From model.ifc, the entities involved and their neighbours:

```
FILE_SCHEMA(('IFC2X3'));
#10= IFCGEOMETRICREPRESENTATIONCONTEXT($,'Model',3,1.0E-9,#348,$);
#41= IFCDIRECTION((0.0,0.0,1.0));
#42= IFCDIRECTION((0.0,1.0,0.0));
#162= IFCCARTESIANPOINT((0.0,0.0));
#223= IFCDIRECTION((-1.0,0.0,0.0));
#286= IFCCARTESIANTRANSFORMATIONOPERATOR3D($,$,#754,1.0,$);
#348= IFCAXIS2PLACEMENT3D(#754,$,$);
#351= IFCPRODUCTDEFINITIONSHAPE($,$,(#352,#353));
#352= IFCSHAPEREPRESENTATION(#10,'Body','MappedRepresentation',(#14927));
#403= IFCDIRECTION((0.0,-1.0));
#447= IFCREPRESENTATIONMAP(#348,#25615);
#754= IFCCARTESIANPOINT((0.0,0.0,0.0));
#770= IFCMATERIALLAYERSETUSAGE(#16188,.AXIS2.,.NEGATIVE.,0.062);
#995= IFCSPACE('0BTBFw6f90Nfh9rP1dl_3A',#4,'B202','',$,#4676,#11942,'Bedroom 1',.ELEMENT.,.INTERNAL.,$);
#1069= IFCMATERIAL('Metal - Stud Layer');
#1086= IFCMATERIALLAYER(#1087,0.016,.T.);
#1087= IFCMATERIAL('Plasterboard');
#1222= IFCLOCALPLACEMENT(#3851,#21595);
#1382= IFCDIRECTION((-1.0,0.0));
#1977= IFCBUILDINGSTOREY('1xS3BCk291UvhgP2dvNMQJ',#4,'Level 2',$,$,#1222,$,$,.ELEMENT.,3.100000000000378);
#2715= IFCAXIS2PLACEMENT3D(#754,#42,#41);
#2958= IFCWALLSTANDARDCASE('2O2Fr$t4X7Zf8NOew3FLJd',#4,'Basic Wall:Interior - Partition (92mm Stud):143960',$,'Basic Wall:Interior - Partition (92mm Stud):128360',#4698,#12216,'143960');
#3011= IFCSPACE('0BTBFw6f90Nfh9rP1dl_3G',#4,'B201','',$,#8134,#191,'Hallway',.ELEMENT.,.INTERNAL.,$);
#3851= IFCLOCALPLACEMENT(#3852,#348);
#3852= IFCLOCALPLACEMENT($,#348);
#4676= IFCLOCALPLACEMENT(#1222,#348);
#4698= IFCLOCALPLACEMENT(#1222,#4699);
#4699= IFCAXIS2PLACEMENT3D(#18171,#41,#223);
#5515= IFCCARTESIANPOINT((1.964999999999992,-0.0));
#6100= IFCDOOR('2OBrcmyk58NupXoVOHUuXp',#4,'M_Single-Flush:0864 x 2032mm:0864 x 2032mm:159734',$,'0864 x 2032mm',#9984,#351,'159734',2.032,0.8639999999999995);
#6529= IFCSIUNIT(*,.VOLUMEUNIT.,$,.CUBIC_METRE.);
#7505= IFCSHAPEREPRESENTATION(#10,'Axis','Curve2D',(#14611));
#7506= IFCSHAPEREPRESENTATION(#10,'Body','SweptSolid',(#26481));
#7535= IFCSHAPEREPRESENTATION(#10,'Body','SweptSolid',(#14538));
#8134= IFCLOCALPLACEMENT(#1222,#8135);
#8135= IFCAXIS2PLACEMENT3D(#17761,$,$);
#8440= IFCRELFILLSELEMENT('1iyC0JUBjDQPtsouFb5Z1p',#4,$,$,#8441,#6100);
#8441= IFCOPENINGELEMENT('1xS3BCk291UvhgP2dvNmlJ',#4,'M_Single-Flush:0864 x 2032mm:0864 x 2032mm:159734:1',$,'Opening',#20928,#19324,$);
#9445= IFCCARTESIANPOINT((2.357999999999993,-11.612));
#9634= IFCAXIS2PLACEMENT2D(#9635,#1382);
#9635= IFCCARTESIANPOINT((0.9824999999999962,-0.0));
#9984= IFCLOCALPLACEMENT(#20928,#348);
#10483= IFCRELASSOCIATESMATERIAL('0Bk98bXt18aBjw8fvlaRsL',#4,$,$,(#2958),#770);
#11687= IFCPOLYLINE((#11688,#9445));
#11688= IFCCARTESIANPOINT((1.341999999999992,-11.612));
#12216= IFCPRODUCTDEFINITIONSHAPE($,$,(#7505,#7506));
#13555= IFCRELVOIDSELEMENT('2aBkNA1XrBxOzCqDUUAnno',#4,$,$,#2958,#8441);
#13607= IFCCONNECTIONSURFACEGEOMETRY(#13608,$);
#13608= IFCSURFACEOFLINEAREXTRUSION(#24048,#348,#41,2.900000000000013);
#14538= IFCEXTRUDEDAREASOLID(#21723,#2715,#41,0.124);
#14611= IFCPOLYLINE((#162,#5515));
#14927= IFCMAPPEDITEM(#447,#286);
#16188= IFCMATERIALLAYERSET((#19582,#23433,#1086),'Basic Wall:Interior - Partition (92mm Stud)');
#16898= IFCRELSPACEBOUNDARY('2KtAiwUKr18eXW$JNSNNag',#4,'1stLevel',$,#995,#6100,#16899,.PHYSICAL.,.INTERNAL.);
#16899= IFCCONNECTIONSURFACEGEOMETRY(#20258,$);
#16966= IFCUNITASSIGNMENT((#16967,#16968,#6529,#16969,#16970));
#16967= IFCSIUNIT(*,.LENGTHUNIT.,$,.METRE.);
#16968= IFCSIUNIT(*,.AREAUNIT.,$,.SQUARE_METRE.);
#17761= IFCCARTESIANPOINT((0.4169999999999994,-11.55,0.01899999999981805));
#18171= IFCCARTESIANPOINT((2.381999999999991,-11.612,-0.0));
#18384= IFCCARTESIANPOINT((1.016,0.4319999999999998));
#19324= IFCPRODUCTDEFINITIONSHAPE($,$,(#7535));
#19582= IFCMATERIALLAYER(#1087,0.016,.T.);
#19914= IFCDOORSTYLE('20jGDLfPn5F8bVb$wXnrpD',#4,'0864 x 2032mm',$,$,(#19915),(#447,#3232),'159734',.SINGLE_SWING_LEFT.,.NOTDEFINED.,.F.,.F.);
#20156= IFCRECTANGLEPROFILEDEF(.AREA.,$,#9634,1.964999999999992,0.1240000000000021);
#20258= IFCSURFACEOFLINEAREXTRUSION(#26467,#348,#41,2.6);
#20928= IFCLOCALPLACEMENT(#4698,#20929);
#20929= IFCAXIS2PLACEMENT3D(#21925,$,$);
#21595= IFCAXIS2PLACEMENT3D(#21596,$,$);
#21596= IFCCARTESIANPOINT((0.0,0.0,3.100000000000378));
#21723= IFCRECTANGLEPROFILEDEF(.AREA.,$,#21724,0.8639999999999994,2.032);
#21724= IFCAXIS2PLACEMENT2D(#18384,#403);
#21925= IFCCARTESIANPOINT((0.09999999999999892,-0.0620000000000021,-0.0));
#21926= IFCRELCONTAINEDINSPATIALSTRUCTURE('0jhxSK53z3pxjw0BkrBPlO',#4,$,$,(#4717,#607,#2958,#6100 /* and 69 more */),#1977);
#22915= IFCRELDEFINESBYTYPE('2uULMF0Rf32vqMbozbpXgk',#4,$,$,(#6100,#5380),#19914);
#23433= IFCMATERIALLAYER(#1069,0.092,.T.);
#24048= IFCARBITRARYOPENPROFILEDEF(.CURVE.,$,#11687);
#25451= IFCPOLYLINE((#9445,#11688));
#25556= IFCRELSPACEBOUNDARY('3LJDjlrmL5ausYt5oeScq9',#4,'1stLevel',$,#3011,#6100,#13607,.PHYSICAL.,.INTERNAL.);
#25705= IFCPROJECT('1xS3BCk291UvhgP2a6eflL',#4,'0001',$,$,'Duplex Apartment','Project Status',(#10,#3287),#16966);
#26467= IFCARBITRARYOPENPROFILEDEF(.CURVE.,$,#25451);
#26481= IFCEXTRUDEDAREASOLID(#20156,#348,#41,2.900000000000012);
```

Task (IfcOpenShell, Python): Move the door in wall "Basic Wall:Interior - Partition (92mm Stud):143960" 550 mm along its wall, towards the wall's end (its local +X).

```python
import numpy as np
import ifcopenshell
import ifcopenshell.api.geometry
import ifcopenshell.util.placement
import ifcopenshell.util.unit

model = ifcopenshell.open("model.ifc")
unit_scale = ifcopenshell.util.unit.calculate_unit_scale(model)

door = model.by_guid("2OBrcmyk58NupXoVOHUuXp")
opening = door.FillsVoids[0].RelatingOpeningElement
wall = opening.VoidsElements[0].RelatingBuildingElement

wall_matrix = ifcopenshell.util.placement.get_local_placement(wall.ObjectPlacement)
shift = wall_matrix[:3, 0] * 0.55 / unit_scale
before = ifcopenshell.util.placement.get_local_placement(door.ObjectPlacement)[:3, 3].copy()

# The door is placed relative to its opening, so it follows when the opening moves.
matrix = ifcopenshell.util.placement.get_local_placement(opening.ObjectPlacement)
matrix[:3, 3] += shift
ifcopenshell.api.geometry.edit_object_placement(
    model, product=opening, matrix=matrix, is_si=False, should_transform_children=True
)

# Space boundary surfaces are stored in each space's coordinates; move them too.
for rel in door.ProvidesBoundaries:
    if not rel.ConnectionGeometry:
        continue
    surface = rel.ConnectionGeometry.SurfaceOnRelatingElement
    space_matrix = ifcopenshell.util.placement.get_local_placement(rel.RelatingSpace.ObjectPlacement)
    point = np.array(surface.Position.Location.Coordinates) + space_matrix[:3, :3].T @ shift
    surface.Position = model.createIfcAxis2Placement3D(
        model.createIfcCartesianPoint(point.tolist()), surface.Position.Axis, surface.Position.RefDirection
    )

after = ifcopenshell.util.placement.get_local_placement(door.ObjectPlacement)[:3, 3]
print("door moved by", (after - before).round(3) + 0.0)

model.write("model_rev.ifc")
```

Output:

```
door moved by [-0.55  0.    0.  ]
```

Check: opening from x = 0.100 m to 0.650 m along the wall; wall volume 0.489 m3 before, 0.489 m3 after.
